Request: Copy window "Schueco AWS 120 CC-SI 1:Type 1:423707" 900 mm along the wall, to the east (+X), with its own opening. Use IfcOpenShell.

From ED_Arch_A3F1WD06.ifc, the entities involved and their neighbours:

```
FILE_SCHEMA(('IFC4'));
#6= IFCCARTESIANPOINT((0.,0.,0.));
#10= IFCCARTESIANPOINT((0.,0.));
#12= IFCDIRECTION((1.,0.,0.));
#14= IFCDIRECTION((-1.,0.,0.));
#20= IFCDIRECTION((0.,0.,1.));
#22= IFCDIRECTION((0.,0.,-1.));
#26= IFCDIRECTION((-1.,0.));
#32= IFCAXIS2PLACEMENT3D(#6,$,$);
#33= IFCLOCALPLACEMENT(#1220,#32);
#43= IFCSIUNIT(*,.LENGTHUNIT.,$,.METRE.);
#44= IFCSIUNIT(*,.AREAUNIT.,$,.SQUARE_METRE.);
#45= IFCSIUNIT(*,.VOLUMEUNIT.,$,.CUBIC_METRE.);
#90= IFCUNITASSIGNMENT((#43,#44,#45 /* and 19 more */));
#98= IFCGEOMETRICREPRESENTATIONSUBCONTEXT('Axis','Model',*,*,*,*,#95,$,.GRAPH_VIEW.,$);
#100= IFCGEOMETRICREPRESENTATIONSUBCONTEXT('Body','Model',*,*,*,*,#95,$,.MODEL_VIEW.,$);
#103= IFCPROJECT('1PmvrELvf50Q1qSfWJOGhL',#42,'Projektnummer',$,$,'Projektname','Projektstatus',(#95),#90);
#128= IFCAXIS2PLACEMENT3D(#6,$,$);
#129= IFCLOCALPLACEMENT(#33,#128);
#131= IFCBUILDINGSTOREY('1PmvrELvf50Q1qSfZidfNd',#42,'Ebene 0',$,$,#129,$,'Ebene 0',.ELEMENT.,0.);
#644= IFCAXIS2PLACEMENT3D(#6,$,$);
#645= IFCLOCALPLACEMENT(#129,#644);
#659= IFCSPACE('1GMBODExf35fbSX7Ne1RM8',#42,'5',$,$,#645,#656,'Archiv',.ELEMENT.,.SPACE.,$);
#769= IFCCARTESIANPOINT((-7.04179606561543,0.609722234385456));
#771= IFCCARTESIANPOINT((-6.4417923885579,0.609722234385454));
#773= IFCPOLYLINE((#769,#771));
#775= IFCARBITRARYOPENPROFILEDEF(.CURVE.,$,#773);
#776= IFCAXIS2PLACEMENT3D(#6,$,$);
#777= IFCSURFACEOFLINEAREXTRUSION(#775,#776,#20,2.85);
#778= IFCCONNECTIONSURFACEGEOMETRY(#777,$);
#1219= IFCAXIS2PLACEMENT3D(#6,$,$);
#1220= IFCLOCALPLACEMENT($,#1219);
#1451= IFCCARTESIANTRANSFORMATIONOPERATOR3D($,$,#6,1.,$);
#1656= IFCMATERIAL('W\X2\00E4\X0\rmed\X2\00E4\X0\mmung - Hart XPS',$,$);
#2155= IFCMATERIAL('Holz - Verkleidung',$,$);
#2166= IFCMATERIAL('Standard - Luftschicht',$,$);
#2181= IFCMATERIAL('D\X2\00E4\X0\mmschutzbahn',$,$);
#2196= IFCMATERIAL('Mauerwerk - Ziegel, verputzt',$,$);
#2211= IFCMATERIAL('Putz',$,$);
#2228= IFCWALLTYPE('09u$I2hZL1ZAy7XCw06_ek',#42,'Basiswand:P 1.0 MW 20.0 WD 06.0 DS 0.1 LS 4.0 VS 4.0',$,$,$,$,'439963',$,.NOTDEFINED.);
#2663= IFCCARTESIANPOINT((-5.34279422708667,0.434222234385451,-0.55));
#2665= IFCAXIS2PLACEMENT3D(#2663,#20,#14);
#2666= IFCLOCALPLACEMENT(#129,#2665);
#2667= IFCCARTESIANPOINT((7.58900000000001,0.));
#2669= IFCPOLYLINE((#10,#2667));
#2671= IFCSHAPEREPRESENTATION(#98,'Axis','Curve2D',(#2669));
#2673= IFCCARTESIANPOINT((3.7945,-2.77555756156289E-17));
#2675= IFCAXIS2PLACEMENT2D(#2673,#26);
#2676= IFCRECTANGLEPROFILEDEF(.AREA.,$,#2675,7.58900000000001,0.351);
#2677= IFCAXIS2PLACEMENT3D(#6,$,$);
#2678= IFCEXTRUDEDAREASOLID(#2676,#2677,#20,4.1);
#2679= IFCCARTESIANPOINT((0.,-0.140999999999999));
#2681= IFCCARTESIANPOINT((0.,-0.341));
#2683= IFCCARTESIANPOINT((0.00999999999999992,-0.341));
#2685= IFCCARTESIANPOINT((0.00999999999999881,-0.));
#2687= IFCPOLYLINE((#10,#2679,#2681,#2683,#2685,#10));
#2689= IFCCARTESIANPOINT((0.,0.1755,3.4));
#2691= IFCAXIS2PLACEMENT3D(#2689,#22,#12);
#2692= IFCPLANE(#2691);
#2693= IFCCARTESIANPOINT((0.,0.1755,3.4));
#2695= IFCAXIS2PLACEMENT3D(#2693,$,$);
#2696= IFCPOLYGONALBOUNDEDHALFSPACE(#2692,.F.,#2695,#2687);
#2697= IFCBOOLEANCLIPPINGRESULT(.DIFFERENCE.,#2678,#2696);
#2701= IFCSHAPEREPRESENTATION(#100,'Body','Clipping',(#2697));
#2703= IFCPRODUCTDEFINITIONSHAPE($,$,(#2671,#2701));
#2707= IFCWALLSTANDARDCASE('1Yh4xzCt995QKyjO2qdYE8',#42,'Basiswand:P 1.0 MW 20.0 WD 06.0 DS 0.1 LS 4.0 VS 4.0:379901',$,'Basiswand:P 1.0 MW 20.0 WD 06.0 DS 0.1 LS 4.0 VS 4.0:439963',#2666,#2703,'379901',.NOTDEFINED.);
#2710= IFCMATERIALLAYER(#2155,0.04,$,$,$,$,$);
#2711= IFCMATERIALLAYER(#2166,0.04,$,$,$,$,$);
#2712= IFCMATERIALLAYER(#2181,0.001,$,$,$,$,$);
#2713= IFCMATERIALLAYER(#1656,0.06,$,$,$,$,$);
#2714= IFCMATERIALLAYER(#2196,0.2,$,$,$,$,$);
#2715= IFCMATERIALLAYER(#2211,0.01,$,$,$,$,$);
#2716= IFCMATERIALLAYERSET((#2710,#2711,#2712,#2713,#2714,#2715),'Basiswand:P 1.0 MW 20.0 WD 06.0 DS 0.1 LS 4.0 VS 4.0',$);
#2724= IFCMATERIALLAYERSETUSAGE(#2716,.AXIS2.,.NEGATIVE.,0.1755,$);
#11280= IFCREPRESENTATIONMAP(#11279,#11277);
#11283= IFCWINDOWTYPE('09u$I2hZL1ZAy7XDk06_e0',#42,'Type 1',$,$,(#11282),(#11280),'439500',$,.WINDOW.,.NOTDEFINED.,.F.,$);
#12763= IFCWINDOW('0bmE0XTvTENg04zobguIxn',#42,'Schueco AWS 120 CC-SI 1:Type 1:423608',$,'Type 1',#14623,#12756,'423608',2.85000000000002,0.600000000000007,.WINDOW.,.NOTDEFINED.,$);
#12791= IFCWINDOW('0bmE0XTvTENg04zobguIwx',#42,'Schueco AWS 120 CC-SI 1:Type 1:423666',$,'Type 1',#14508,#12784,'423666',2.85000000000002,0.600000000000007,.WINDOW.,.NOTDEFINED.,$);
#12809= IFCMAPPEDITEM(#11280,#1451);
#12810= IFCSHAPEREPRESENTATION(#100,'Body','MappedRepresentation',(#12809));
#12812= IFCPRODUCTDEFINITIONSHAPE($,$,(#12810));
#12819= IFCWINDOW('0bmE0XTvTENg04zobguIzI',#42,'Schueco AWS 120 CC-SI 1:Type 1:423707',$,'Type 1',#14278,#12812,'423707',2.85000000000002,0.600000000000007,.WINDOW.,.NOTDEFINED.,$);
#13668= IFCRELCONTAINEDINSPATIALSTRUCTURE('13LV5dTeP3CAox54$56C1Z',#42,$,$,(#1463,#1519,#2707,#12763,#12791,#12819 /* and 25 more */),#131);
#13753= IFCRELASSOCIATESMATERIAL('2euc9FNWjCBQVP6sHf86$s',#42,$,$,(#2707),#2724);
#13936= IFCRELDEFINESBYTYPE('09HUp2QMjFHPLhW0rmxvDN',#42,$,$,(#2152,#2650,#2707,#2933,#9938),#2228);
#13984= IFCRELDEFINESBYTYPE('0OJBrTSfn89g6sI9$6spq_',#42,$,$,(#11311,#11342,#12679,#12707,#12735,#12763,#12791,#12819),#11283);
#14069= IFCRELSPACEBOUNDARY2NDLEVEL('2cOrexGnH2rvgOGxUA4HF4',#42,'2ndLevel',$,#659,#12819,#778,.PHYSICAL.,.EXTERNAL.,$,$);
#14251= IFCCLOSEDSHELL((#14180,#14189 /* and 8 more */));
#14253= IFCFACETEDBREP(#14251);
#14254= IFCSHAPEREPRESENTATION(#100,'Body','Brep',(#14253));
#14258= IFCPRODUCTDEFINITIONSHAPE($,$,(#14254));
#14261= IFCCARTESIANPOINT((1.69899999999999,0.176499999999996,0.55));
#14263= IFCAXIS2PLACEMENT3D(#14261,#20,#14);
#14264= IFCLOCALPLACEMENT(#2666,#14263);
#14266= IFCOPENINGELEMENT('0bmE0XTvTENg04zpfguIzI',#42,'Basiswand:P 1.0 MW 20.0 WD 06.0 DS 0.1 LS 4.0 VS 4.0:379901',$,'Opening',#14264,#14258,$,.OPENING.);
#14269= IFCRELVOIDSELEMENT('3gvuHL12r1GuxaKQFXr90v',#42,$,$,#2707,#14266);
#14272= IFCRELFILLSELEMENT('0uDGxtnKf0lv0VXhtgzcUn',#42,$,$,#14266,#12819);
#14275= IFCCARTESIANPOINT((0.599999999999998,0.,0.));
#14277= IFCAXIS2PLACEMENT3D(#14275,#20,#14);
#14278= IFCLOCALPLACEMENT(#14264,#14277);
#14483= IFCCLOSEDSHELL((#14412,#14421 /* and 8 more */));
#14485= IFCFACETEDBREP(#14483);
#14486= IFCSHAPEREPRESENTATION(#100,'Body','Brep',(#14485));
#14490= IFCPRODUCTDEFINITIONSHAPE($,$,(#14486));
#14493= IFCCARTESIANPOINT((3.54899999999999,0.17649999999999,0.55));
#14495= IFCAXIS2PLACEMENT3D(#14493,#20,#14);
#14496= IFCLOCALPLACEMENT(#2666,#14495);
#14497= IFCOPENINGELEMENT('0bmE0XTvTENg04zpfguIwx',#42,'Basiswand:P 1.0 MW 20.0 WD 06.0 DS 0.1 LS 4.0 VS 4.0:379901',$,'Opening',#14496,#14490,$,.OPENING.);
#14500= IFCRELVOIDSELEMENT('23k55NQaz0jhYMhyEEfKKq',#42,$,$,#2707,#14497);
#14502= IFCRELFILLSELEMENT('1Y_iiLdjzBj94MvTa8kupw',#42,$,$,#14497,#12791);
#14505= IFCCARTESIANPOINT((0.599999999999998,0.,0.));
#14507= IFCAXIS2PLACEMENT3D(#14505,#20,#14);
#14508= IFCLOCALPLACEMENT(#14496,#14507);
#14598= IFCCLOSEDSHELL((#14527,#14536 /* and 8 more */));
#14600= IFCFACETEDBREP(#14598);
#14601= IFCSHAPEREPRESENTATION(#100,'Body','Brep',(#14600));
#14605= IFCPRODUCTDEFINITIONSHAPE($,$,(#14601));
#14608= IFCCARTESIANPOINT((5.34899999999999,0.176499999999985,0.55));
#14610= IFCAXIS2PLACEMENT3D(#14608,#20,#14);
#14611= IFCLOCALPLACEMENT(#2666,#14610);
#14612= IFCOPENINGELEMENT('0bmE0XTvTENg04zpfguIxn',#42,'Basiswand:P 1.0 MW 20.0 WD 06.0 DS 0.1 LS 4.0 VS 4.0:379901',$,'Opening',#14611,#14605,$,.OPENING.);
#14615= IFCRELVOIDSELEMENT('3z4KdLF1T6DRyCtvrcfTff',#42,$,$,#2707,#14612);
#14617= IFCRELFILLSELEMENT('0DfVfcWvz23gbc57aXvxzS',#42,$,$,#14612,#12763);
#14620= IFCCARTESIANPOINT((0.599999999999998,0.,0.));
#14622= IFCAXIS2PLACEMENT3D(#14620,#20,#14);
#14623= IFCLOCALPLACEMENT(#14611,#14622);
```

```python
import numpy as np
import ifcopenshell
import ifcopenshell.api.feature
import ifcopenshell.api.geometry
import ifcopenshell.api.root
import ifcopenshell.geom
import ifcopenshell.util.element
import ifcopenshell.util.placement
import ifcopenshell.util.shape

model = ifcopenshell.open("ED_Arch_A3F1WD06.ifc")
settings = ifcopenshell.geom.settings()


def volume(element):
    """Net volume in cubic metres, openings subtracted."""
    shape = ifcopenshell.geom.create_shape(settings, element)
    return ifcopenshell.util.shape.get_volume(shape.geometry)


def reuse_history(source, copy):
    """copy_class also copies each property set's owner history, people and application; keep the originals."""
    for rel in copy.IsDefinedBy:
        if rel.is_a("IfcRelDefinesByProperties") and (history := rel.RelatingPropertyDefinition.OwnerHistory):
            rel.RelatingPropertyDefinition.OwnerHistory = source.OwnerHistory
            ifcopenshell.util.element.remove_deep2(model, history)


window = model.by_guid("0bmE0XTvTENg04zobguIzI")
opening = window.FillsVoids[0].RelatingOpeningElement
wall = opening.VoidsElements[0].RelatingBuildingElement
before = volume(wall)
shift = ifcopenshell.util.placement.get_local_placement(wall.ObjectPlacement)[:3, 0] * -0.9

# copy_class copies the void relationship, type, container and properties, but no geometry.
new_opening = ifcopenshell.api.root.copy_class(model, product=opening)
new_opening.Representation = ifcopenshell.util.element.copy_deep(
    model, opening.Representation, exclude=["IfcGeometricRepresentationContext", "IfcRepresentationMap"]
)
new_opening.Name = "Basiswand:P 1.0 MW 20.0 WD 06.0 DS 0.1 LS 4.0 VS 4.0"
new_window = ifcopenshell.api.root.copy_class(model, product=window)
new_window.Representation = ifcopenshell.util.element.copy_deep(
    model, window.Representation, exclude=["IfcGeometricRepresentationContext", "IfcRepresentationMap"]
)
new_window.Name = "Schueco AWS 120 CC-SI 1:Type 1"
new_window.Tag = None
reuse_history(window, new_window)
ifcopenshell.api.feature.add_filling(model, opening=new_opening, element=new_window)

for old, new in ((opening, new_opening), (window, new_window)):
    matrix = ifcopenshell.util.placement.get_local_placement(old.ObjectPlacement)
    matrix[:3, 3] += shift
    ifcopenshell.api.geometry.edit_object_placement(model, product=new, matrix=matrix, is_si=False)

# The copied space boundaries still share their surfaces with the original.
for rel in new_window.ProvidesBoundaries:
    if rel.ConnectionGeometry:
        rel.ConnectionGeometry = ifcopenshell.util.element.copy_deep(model, rel.ConnectionGeometry)

# Space boundary surfaces are stored in each space's coordinates; move them too.
for rel in new_window.ProvidesBoundaries:
    if not rel.ConnectionGeometry:
        continue
    surface = rel.ConnectionGeometry.SurfaceOnRelatingElement
    space_matrix = ifcopenshell.util.placement.get_local_placement(rel.RelatingSpace.ObjectPlacement)
    point = np.array(surface.Position.Location.Coordinates) + space_matrix[:3, :3].T @ shift
    surface.Position = model.createIfcAxis2Placement3D(
        model.createIfcCartesianPoint(point.tolist()), surface.Position.Axis, surface.Position.RefDirection
    )

after = volume(wall)

print(f"wall volume {before:.3f} -> {after:.3f} m3")

model.write("ED_Arch_A3F1WD06_edited.ifc")
```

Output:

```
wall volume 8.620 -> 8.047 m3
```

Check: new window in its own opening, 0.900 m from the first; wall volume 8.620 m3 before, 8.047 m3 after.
